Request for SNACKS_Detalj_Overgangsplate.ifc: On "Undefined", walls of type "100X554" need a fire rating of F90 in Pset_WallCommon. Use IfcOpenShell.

First a look at what the model holds.

```python
import ifcopenshell
import ifcopenshell.util.element

model = ifcopenshell.open("SNACKS_Detalj_Overgangsplate.ifc")
print(model.schema)
storey = next(s for s in model.by_type("IfcBuildingStorey") if s.Name == "Undefined")
walls = [e for e in ifcopenshell.util.element.get_decomposition(storey) if e.is_a("IfcWall")]
seen = {}
for e in walls:
    element_type = ifcopenshell.util.element.get_type(e)
    key = (element_type.Name if element_type != e and element_type else None, ifcopenshell.util.element.get_pset(e, "Pset_WallCommon", "FireRating"))
    seen[key] = seen.get(key, 0) + 1
for (name, value), count in sorted(seen.items(), key=str):
    print(count, "x", name, "|", value)
```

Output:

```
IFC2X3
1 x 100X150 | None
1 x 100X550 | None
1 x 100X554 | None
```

```python
import ifcopenshell
import ifcopenshell.api.pset
import ifcopenshell.util.element

model = ifcopenshell.open("SNACKS_Detalj_Overgangsplate.ifc")

storey = next(s for s in model.by_type("IfcBuildingStorey") if s.Name == "Undefined")
walls = [e for e in ifcopenshell.util.element.get_decomposition(storey) if e.is_a("IfcWall")]

count = 0
for e in walls:
    element_type = ifcopenshell.util.element.get_type(e)
    if element_type in (None, e) or element_type.Name != "100X554":
        continue
    # add_pset returns the element's existing set when there is one.
    pset = ifcopenshell.api.pset.add_pset(model, product=e, name="Pset_WallCommon")
    ifcopenshell.api.pset.edit_pset(model, pset=pset, properties={"FireRating": "F90"})
    count += 1

print(count, "walls updated")

model.write("SNACKS_Detalj_Overgangsplate-out.ifc")
```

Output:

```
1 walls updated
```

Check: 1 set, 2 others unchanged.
